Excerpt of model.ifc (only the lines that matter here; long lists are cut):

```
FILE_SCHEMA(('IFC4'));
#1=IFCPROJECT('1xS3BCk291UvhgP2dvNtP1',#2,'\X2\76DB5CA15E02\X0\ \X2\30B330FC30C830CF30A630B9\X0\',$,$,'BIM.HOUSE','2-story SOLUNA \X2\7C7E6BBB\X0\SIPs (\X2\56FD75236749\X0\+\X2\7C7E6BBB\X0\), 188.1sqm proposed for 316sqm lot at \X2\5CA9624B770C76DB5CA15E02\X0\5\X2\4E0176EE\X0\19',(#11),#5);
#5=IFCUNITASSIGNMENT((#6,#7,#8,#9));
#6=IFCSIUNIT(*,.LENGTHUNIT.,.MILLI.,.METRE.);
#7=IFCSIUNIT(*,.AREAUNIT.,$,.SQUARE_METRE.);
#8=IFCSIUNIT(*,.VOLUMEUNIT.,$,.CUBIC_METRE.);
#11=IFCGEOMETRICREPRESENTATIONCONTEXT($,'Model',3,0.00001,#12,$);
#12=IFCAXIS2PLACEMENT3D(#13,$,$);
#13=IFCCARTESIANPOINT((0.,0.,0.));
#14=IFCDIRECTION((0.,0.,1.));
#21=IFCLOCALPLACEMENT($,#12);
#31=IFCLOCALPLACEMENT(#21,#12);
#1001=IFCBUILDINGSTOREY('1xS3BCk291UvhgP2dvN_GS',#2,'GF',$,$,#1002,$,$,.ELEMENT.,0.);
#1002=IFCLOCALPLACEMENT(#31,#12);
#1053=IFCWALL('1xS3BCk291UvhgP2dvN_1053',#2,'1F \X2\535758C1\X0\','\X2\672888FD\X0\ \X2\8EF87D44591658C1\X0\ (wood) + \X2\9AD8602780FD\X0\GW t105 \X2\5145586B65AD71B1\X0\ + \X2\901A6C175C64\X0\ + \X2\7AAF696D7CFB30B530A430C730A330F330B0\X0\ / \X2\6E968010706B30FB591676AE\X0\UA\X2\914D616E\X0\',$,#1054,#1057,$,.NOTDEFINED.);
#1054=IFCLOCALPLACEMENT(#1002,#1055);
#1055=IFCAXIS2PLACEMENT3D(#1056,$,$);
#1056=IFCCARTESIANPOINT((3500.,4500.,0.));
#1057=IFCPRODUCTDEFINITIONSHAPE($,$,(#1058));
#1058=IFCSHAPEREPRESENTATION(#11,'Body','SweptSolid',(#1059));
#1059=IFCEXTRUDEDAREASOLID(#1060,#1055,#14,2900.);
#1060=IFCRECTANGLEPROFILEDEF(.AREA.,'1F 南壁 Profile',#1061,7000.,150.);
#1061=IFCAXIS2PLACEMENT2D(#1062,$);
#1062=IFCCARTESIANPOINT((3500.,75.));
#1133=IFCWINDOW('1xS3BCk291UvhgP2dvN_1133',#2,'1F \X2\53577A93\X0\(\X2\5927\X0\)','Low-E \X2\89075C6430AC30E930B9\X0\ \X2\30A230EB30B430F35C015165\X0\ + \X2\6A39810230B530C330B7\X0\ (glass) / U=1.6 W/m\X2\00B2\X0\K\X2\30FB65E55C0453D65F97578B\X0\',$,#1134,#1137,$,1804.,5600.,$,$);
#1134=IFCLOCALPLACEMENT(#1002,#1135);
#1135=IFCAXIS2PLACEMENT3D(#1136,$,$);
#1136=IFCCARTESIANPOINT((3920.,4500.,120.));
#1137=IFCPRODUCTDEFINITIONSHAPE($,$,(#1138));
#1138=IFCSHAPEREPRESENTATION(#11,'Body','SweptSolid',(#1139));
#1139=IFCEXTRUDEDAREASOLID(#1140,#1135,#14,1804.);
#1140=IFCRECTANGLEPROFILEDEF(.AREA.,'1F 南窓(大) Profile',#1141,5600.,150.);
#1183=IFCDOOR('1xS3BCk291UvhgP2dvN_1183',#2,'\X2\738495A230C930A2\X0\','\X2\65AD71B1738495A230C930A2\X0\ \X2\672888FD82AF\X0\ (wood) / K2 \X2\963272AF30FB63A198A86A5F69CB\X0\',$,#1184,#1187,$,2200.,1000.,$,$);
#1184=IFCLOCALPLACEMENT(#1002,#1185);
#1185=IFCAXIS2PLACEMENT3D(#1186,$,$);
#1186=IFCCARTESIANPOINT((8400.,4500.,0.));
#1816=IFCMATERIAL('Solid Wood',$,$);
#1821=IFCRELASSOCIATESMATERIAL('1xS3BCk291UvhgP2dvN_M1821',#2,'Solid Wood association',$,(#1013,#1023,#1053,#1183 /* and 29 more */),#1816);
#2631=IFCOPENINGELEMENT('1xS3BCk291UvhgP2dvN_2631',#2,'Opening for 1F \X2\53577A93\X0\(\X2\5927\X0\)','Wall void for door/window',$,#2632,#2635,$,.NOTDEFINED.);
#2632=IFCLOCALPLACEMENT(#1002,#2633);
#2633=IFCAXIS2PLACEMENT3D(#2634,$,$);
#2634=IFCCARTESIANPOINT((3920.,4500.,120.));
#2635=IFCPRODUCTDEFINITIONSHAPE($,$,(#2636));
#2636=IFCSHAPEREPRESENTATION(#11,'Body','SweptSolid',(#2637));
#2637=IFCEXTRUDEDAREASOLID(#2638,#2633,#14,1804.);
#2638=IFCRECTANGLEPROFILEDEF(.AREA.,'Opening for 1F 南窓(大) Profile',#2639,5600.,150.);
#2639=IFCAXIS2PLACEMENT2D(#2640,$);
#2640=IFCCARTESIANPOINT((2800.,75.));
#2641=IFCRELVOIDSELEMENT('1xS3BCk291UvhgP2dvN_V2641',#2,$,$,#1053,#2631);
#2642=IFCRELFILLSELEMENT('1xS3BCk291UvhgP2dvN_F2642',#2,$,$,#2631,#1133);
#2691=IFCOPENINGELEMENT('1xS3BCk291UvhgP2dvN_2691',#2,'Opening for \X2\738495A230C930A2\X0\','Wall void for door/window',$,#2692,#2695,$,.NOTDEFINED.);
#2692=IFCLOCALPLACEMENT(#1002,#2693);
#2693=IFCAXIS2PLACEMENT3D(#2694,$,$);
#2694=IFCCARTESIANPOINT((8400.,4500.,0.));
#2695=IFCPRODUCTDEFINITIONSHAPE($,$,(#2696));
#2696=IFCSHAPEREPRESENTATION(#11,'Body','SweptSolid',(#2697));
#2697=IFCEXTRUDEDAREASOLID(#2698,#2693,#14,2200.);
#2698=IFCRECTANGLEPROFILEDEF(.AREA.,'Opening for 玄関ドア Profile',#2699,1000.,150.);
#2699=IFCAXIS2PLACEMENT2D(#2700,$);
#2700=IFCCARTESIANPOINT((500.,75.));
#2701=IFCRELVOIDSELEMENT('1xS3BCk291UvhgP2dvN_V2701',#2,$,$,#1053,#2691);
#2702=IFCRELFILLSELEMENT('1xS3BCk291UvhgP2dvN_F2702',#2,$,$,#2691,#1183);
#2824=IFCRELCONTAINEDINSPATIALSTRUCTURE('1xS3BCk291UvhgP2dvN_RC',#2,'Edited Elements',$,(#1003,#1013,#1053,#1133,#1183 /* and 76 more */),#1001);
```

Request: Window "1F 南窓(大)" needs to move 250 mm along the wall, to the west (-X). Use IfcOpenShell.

```python
import ifcopenshell
import ifcopenshell.api.geometry
import ifcopenshell.util.placement

model = ifcopenshell.open("model.ifc")

window = model.by_guid("1xS3BCk291UvhgP2dvN_1133")
opening = window.FillsVoids[0].RelatingOpeningElement
wall = opening.VoidsElements[0].RelatingBuildingElement

wall_matrix = ifcopenshell.util.placement.get_local_placement(wall.ObjectPlacement)
shift = wall_matrix[:3, 0] * -250.0
before = ifcopenshell.util.placement.get_local_placement(window.ObjectPlacement)[:3, 3].copy()

# The window is not placed relative to its opening, so move both.
for product in (opening, window):
    matrix = ifcopenshell.util.placement.get_local_placement(product.ObjectPlacement)
    matrix[:3, 3] += shift
    ifcopenshell.api.geometry.edit_object_placement(model, product=product, matrix=matrix, is_si=False)

after = ifcopenshell.util.placement.get_local_placement(window.ObjectPlacement)[:3, 3]
print("window moved by", (after - before).round(3) + 0.0)

model.write("model_edited.ifc")
```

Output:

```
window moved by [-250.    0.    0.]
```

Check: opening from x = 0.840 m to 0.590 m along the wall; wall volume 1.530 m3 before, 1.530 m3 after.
